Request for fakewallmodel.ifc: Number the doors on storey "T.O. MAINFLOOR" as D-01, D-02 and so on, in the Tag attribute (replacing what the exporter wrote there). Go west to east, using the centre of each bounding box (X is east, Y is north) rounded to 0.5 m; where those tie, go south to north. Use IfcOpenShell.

First a look at what the model holds.

```python
import ifcopenshell
import ifcopenshell.util.element
import ifcopenshell.util.placement

model = ifcopenshell.open("fakewallmodel.ifc")
print(model.schema)
storey = next(s for s in model.by_type("IfcBuildingStorey") if s.Name == "T.O. MAINFLOOR")
doors = [e for e in ifcopenshell.util.element.get_decomposition(storey) if e.is_a("IfcDoor")]
for e in sorted(doors, key=lambda e: e.id()):
    origin = ifcopenshell.util.placement.get_local_placement(e.ObjectPlacement)[:3, 3]
    print(e.id(), e.Tag, e.Name, origin.round(2) + 0.0, sep=" | ")
```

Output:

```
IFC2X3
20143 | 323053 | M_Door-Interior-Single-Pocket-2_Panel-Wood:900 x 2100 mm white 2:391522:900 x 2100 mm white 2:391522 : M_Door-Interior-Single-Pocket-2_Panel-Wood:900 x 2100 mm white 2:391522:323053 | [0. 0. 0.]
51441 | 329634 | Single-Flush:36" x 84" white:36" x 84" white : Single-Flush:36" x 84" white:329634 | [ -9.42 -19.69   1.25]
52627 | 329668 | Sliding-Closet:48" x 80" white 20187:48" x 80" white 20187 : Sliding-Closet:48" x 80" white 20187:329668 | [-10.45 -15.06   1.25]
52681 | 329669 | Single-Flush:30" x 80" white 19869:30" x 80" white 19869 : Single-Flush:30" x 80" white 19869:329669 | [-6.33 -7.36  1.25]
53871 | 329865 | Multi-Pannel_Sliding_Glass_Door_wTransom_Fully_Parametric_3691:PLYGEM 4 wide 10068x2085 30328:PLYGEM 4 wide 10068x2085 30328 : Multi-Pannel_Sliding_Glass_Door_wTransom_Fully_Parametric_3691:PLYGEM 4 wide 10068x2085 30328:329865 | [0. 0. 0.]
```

```python
import ifcopenshell
import ifcopenshell.geom
import ifcopenshell.util.element
import ifcopenshell.util.shape

model = ifcopenshell.open("fakewallmodel.ifc")
settings = ifcopenshell.geom.settings()
settings.set("use-world-coords", True)


def centre(element):
    shape = ifcopenshell.geom.create_shape(settings, element)
    return ifcopenshell.util.shape.get_bbox_centroid(shape.geometry)


storey = next(s for s in model.by_type("IfcBuildingStorey") if s.Name == "T.O. MAINFLOOR")
doors = [e for e in ifcopenshell.util.element.get_decomposition(storey) if e.is_a("IfcDoor")]

# Insertion points can sit at a corner or the storey origin, so sort by the geometry (in metres).
centres = {e: centre(e) for e in doors}
doors.sort(key=lambda e: (round(centres[e][0] / 0.5), centres[e][1]))

for i, e in enumerate(doors, start=1):
    number = f"D-{i:02d}"
    e.Tag = number
    print(e.id(), number)

model.write("fakewallmodel_rev.ifc")
```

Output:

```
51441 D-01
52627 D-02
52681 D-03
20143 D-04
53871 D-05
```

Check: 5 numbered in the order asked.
